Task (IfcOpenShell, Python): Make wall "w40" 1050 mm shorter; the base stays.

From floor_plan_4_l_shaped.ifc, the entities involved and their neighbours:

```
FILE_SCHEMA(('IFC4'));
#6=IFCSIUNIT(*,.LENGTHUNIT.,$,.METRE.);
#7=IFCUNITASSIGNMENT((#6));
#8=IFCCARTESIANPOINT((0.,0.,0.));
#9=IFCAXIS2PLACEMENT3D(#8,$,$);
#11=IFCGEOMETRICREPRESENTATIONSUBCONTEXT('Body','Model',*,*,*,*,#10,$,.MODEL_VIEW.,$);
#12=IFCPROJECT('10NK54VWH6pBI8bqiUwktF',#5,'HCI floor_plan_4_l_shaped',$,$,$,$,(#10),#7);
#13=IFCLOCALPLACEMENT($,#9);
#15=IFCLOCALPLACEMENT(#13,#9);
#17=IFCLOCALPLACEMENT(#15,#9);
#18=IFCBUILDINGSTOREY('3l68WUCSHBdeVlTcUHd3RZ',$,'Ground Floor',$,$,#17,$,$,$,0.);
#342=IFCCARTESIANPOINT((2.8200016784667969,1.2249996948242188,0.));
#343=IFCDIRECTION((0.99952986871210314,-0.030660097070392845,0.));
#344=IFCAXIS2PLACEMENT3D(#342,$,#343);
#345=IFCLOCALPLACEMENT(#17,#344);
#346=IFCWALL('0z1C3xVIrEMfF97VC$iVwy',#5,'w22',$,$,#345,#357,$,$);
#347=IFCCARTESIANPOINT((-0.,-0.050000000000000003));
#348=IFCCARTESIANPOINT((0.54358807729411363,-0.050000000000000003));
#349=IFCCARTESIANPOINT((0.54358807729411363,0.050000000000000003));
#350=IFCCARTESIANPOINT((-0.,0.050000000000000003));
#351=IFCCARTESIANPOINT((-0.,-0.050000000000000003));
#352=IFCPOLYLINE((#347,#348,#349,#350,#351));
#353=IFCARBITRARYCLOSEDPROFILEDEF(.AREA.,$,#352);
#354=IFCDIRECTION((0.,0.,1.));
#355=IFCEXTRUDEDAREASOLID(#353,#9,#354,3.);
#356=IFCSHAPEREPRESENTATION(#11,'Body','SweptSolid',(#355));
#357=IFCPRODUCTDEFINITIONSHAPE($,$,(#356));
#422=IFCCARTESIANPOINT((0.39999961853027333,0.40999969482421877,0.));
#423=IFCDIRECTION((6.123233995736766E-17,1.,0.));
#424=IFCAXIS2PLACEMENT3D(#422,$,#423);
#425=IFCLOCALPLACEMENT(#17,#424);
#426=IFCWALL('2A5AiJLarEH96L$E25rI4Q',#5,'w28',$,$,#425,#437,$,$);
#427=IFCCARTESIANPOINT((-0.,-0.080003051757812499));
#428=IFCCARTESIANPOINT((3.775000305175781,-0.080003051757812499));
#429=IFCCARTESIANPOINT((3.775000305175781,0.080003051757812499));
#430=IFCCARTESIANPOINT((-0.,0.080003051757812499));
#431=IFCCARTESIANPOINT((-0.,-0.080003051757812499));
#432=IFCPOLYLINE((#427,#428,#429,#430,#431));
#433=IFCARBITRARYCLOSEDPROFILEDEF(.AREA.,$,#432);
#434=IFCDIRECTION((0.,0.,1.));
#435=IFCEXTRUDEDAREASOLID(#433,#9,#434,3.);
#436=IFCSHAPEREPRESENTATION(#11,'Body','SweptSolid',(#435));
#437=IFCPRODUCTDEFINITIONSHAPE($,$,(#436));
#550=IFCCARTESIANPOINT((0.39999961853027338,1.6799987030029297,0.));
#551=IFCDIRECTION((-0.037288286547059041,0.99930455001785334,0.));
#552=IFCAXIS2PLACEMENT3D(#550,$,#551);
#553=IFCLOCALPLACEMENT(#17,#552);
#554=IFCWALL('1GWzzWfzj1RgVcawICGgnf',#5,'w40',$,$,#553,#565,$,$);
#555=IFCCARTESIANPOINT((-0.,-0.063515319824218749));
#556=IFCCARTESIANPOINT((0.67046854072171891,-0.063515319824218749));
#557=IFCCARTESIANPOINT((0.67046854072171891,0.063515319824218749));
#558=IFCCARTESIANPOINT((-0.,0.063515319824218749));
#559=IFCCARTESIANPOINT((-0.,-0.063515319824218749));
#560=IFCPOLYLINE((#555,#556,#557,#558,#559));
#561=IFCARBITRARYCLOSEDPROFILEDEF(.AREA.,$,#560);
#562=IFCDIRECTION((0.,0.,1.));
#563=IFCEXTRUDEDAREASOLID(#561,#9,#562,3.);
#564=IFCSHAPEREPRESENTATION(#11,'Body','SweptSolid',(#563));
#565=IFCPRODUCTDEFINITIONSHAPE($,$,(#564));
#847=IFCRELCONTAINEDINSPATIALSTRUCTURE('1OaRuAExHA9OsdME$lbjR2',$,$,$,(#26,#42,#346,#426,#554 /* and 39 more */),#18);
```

```python
import ifcopenshell
import ifcopenshell.geom
import ifcopenshell.util.representation
import ifcopenshell.util.shape

model = ifcopenshell.open("floor_plan_4_l_shaped.ifc")
settings = ifcopenshell.geom.settings()


def volume(element):
    """Net volume in cubic metres, openings subtracted."""
    shape = ifcopenshell.geom.create_shape(settings, element)
    return ifcopenshell.util.shape.get_volume(shape.geometry)


wall = model.by_guid("1GWzzWfzj1RgVcawICGgnf")
before = volume(wall)

body = ifcopenshell.util.representation.get_representation(wall, "Model", "Body")
solid = body.Items[0]
old_height = solid.Depth
solid.Depth -= 1.05
after = volume(wall)

print(f"height {old_height:g} -> {solid.Depth:g}, volume {before:.3f} -> {after:.3f} m3")

model.write("floor_plan_4_l_shaped_rev.ifc")
```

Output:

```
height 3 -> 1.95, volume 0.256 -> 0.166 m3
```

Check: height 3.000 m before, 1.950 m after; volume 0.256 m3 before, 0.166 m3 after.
